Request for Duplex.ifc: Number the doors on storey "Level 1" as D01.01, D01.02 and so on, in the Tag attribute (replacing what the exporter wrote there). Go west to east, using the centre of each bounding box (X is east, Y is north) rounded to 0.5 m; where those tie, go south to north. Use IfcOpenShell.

First a look at what the model holds.

```python
import ifcopenshell
import ifcopenshell.util.element
import ifcopenshell.util.placement

model = ifcopenshell.open("Duplex.ifc")
print(model.schema)
storey = next(s for s in model.by_type("IfcBuildingStorey") if s.Name == "Level 1")
doors = [e for e in ifcopenshell.util.element.get_decomposition(storey) if e.is_a("IfcDoor")]
for e in sorted(doors, key=lambda e: e.id()):
    origin = ifcopenshell.util.placement.get_local_placement(e.ObjectPlacement)[:3, 3]
    print(e.id(), e.Tag, e.Name, origin.round(2) + 0.0, sep=" | ")
```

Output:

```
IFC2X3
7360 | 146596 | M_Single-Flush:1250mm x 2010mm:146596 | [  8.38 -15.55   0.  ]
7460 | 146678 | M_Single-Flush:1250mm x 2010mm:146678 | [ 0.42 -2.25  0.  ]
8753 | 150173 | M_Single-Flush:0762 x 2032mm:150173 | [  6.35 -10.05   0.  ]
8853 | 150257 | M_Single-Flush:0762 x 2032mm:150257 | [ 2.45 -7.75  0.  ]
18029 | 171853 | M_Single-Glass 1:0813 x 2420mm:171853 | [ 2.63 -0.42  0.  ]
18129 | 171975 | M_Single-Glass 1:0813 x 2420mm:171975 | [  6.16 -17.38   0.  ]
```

```python
import ifcopenshell
import ifcopenshell.geom
import ifcopenshell.util.element
import ifcopenshell.util.shape

model = ifcopenshell.open("Duplex.ifc")
settings = ifcopenshell.geom.settings()
settings.set("use-world-coords", True)


def centre(element):
    shape = ifcopenshell.geom.create_shape(settings, element)
    return ifcopenshell.util.shape.get_bbox_centroid(shape.geometry)


storey = next(s for s in model.by_type("IfcBuildingStorey") if s.Name == "Level 1")
doors = [e for e in ifcopenshell.util.element.get_decomposition(storey) if e.is_a("IfcDoor")]

# Insertion points can sit at a corner or the storey origin, so sort by the geometry (in metres).
centres = {e: centre(e) for e in doors}
doors.sort(key=lambda e: (round(centres[e][0] / 0.5), centres[e][1]))

for i, e in enumerate(doors, start=1):
    number = f"D01.{i:02d}"
    e.Tag = number
    print(e.id(), number)

model.write("Duplex_rev.ifc")
```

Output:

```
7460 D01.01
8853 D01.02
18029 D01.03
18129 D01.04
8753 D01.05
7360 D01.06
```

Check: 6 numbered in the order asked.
